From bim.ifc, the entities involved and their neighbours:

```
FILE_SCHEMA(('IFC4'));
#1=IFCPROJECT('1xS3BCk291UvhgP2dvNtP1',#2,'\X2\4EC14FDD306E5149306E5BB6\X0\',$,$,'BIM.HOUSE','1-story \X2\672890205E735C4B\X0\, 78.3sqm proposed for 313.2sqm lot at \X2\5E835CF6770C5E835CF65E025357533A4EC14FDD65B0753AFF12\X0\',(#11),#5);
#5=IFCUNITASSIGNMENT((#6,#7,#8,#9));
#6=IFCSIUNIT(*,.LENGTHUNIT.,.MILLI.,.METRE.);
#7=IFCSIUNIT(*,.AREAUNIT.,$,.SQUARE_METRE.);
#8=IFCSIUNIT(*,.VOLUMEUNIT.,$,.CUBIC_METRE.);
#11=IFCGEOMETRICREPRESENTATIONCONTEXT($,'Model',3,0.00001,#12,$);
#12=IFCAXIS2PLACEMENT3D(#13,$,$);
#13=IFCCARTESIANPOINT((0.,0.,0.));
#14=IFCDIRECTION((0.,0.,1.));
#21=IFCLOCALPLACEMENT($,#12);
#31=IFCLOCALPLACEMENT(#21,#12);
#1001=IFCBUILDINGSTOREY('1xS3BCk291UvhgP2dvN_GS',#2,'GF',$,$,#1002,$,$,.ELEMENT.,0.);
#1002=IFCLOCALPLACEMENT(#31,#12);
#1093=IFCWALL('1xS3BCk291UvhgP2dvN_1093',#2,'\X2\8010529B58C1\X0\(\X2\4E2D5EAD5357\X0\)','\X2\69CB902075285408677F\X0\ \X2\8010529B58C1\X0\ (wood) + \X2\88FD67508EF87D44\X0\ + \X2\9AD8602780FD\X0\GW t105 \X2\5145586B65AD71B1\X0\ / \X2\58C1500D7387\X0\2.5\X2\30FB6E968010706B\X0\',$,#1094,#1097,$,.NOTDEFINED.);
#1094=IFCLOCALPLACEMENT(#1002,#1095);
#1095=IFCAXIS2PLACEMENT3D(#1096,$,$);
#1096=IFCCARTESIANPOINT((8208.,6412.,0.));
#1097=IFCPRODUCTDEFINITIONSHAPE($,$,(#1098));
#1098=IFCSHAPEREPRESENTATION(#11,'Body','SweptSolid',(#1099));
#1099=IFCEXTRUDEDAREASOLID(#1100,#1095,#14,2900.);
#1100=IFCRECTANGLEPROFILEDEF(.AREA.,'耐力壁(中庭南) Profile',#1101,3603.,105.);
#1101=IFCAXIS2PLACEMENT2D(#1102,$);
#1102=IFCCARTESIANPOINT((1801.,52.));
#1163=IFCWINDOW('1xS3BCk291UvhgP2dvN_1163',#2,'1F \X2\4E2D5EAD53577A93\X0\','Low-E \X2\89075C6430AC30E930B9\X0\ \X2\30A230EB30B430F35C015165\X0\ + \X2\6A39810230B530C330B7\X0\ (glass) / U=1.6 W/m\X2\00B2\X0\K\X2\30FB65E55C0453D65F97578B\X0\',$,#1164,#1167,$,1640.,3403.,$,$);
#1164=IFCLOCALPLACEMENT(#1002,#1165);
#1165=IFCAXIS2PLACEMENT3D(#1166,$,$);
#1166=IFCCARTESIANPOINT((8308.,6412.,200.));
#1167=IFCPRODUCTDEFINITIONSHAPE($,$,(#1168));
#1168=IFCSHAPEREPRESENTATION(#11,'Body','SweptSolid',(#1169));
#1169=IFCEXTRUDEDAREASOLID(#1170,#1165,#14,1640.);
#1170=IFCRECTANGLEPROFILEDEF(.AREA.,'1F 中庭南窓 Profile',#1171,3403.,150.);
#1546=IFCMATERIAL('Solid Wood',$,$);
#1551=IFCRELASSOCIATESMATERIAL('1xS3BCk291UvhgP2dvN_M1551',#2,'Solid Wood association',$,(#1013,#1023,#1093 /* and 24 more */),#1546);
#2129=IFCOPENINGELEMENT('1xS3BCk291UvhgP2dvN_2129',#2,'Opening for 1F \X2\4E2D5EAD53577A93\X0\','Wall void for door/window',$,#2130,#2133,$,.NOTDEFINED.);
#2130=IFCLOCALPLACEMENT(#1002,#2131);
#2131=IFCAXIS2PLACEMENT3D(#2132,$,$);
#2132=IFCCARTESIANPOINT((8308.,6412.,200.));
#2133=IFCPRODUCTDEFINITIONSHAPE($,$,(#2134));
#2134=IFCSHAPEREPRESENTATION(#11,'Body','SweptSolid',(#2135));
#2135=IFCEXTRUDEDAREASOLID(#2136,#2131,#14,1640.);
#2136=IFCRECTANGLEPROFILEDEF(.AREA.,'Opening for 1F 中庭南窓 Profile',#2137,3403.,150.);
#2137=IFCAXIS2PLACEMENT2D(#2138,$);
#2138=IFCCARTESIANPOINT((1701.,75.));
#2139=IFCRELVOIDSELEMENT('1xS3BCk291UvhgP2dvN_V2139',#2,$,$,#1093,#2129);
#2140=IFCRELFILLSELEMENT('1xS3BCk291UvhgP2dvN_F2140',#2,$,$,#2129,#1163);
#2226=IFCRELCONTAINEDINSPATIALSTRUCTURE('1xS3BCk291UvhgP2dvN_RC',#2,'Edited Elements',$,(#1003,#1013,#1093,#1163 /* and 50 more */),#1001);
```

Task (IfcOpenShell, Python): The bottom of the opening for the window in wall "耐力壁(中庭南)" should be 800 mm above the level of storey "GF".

```python
import numpy as np
import ifcopenshell
import ifcopenshell.api.geometry
import ifcopenshell.geom
import ifcopenshell.util.element
import ifcopenshell.util.placement
import ifcopenshell.util.shape
import ifcopenshell.util.unit

model = ifcopenshell.open("bim.ifc")
unit_scale = ifcopenshell.util.unit.calculate_unit_scale(model)

window = model.by_guid("1xS3BCk291UvhgP2dvN_1163")
opening = window.FillsVoids[0].RelatingOpeningElement
storey = ifcopenshell.util.element.get_container(window, ifc_class="IfcBuildingStorey")
level = ifcopenshell.util.placement.get_local_placement(storey.ObjectPlacement)[2, 3]

# The opening's origin need not be at the sill, so measure its lowest point.
shape = ifcopenshell.geom.create_shape(ifcopenshell.geom.settings(), opening)
bottom = ifcopenshell.util.shape.get_shape_bottom_elevation(shape, shape.geometry) / unit_scale
dz = level + 0.8 / unit_scale - bottom

shift = np.array([0.0, 0.0, dz])
# The window is not placed relative to its opening, so move both.
for product in (opening, window):
    matrix = ifcopenshell.util.placement.get_local_placement(product.ObjectPlacement)
    matrix[:3, 3] += shift
    ifcopenshell.api.geometry.edit_object_placement(model, product=product, matrix=matrix, is_si=False)

print(f"moved by {dz * unit_scale:+.3f} m")

model.write("bim_updated.ifc")
```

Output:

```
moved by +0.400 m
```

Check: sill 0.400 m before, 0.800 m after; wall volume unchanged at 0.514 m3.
